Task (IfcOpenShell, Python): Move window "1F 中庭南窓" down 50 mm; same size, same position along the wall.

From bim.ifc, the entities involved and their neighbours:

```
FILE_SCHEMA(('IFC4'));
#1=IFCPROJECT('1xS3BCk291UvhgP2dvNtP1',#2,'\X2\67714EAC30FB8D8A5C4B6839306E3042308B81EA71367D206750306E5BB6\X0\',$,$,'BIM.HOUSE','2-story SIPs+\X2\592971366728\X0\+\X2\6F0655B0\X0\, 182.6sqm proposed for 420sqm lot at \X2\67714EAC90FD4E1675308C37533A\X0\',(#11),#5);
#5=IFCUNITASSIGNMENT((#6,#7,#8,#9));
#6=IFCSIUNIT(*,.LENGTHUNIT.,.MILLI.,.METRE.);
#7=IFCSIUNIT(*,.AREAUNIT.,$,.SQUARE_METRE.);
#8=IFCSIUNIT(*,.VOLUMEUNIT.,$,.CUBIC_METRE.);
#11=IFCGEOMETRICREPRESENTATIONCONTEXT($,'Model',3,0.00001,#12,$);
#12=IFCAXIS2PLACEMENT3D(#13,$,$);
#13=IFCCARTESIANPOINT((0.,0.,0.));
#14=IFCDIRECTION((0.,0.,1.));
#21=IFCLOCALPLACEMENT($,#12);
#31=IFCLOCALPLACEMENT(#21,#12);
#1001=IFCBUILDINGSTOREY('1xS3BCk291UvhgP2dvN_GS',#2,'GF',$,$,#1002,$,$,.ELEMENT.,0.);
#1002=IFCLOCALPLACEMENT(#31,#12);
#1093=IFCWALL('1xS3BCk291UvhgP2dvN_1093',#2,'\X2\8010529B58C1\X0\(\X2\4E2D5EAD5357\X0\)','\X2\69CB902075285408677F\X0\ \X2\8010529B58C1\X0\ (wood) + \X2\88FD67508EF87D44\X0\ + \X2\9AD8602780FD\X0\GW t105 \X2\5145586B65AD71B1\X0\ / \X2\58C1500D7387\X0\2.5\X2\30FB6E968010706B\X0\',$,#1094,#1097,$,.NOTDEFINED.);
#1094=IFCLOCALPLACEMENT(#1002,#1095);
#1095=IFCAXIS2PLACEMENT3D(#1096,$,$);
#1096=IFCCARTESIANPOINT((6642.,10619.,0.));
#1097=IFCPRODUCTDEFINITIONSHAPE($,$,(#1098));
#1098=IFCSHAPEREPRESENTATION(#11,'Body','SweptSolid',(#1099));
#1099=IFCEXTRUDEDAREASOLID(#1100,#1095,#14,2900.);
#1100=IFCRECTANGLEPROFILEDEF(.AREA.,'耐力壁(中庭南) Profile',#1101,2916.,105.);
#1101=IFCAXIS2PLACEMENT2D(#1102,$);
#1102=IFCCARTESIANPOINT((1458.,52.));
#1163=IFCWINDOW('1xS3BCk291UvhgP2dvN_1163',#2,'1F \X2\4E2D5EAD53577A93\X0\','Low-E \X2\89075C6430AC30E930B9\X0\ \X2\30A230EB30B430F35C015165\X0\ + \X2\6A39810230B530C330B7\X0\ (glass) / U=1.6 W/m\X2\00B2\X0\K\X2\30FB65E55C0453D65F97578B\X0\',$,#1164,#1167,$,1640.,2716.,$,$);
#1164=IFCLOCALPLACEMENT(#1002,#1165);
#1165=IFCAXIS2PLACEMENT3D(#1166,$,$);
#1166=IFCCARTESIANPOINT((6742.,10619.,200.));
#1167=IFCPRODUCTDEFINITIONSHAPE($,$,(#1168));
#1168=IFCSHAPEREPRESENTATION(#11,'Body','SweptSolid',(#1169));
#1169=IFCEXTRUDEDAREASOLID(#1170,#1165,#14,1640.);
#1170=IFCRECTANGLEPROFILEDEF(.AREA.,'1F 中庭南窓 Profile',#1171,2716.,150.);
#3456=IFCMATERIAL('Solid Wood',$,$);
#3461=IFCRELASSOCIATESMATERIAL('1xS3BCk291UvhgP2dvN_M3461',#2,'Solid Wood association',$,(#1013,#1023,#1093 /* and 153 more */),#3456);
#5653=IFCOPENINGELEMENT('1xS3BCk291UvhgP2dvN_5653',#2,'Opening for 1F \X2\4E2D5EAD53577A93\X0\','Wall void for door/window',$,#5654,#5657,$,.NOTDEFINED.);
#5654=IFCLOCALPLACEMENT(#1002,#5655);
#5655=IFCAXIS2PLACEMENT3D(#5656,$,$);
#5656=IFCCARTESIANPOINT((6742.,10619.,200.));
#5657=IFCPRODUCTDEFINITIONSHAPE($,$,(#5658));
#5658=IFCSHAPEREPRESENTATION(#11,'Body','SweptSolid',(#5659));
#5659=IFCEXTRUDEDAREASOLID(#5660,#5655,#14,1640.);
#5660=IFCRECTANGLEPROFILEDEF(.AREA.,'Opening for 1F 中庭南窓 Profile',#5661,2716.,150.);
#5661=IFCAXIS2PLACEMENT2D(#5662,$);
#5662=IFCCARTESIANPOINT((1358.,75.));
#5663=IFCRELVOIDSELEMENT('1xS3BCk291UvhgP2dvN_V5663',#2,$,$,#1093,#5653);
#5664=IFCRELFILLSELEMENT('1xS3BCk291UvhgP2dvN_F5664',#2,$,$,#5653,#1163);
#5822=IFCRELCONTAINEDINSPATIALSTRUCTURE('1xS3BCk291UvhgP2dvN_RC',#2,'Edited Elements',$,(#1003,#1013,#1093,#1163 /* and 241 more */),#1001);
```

```python
import numpy as np
import ifcopenshell
import ifcopenshell.api.geometry
import ifcopenshell.util.placement
import ifcopenshell.util.unit

model = ifcopenshell.open("bim.ifc")
unit_scale = ifcopenshell.util.unit.calculate_unit_scale(model)

window = model.by_id(1163)
opening = window.FillsVoids[0].RelatingOpeningElement
dz = -0.05 / unit_scale

shift = np.array([0.0, 0.0, dz])
# The window is not placed relative to its opening, so move both.
for product in (opening, window):
    matrix = ifcopenshell.util.placement.get_local_placement(product.ObjectPlacement)
    matrix[:3, 3] += shift
    ifcopenshell.api.geometry.edit_object_placement(model, product=product, matrix=matrix, is_si=False)

print(f"moved by {dz * unit_scale:+.3f} m")

model.write("bim-out.ifc")
```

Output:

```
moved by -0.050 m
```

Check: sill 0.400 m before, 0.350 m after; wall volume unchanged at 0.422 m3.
